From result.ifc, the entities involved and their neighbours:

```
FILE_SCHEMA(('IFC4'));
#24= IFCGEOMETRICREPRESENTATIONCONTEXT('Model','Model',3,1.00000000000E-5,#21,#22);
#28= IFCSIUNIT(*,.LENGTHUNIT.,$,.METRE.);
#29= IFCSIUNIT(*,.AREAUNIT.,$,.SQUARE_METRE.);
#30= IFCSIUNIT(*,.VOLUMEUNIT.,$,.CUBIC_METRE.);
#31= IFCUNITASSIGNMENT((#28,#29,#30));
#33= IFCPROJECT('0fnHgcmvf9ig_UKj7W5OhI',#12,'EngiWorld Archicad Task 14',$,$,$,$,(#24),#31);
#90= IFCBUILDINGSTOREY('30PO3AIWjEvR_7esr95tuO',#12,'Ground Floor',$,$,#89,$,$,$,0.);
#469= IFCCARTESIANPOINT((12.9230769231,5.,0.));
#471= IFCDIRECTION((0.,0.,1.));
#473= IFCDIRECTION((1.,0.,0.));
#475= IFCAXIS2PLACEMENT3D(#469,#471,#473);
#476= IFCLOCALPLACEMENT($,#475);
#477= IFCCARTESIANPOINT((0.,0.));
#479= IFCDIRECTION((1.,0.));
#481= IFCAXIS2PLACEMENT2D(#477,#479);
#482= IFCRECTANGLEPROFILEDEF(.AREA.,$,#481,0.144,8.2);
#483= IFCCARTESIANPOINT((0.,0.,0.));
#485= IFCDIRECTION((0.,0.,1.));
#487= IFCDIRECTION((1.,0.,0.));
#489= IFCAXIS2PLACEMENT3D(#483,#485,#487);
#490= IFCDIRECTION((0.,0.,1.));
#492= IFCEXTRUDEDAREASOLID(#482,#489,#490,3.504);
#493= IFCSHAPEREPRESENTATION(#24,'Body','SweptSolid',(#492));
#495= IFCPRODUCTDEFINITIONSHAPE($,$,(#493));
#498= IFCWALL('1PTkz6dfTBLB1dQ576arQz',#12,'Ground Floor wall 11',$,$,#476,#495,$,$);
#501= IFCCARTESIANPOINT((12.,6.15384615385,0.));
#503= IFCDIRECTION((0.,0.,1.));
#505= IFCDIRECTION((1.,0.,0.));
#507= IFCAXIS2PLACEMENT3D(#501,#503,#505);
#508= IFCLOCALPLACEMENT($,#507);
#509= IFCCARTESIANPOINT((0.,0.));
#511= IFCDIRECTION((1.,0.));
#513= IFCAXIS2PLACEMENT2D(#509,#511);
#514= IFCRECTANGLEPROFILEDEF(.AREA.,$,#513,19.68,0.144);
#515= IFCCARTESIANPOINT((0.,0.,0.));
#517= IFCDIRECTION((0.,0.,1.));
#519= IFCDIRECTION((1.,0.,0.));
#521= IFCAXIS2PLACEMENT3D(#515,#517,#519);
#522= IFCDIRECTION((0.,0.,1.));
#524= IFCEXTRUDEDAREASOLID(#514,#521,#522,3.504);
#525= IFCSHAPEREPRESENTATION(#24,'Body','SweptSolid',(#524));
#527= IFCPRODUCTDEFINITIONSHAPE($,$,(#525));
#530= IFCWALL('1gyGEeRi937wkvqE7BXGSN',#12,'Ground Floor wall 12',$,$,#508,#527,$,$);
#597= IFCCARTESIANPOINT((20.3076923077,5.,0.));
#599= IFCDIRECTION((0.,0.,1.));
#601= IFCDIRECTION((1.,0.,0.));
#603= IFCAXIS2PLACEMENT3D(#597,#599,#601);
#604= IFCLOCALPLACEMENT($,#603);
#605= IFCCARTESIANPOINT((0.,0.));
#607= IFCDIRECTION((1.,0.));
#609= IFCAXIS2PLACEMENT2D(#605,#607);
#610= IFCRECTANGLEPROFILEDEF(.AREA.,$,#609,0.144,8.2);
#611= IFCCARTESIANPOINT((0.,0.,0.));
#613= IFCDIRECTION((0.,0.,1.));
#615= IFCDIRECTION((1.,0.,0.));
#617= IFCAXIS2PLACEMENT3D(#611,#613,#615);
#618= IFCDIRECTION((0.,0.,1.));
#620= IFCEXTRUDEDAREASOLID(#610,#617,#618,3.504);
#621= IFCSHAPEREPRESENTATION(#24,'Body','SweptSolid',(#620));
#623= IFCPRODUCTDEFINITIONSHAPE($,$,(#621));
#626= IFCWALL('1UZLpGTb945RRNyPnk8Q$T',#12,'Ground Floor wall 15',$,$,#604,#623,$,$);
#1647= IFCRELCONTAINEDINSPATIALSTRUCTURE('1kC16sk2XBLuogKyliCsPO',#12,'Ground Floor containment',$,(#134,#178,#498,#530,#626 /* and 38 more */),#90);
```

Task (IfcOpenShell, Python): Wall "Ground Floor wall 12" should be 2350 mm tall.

```python
import ifcopenshell
import ifcopenshell.geom
import ifcopenshell.util.shape
import ifcopenshell.util.unit

model = ifcopenshell.open("result.ifc")
unit_scale = ifcopenshell.util.unit.calculate_unit_scale(model)
settings = ifcopenshell.geom.settings()


def volume(element):
    """Net volume in cubic metres, openings subtracted."""
    shape = ifcopenshell.geom.create_shape(settings, element)
    return ifcopenshell.util.shape.get_volume(shape.geometry)


wall = model.by_guid("1gyGEeRi937wkvqE7BXGSN")
before = volume(wall)

body = next(r for r in wall.Representation.Representations if r.RepresentationIdentifier == "Body")
solid = body.Items[0]
old_height = solid.Depth
solid.Depth = 2.35 / unit_scale
after = volume(wall)

print(f"height {old_height:g} -> {solid.Depth:g}, volume {before:.3f} -> {after:.3f} m3")

model.write("result_edited.ifc")
```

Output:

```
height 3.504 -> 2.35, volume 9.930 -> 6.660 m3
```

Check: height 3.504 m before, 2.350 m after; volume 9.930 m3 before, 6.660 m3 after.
